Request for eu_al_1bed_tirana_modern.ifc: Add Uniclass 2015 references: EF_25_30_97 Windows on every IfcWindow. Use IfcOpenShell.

First a look at what the model holds.

```python
import ifcopenshell

model = ifcopenshell.open("eu_al_1bed_tirana_modern.ifc")
print(model.schema)
print("classifications:", [c.Name for c in model.by_type("IfcClassification")])
for ifc_class in ("IfcDoor", "IfcRoof", "IfcStair", "IfcWall", "IfcWindow"):
    print(ifc_class, len(model.by_type(ifc_class)))
```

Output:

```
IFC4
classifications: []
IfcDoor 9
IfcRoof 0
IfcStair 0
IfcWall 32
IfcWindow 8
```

```python
import ifcopenshell
import ifcopenshell.api.classification

model = ifcopenshell.open("eu_al_1bed_tirana_modern.ifc")

system = ifcopenshell.api.classification.add_classification(model, classification="Uniclass 2015")

codes = {
    "IfcWindow": ("EF_25_30_97", "Windows"),
}
for ifc_class, (code, name) in codes.items():
    products = model.by_type(ifc_class)
    ifcopenshell.api.classification.add_reference(
        model, products=products, classification=system, identification=code, name=name
    )
    print(code, len(products))

model.write("eu_al_1bed_tirana_modern_v2.ifc")
```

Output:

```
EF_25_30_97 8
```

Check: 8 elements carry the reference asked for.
